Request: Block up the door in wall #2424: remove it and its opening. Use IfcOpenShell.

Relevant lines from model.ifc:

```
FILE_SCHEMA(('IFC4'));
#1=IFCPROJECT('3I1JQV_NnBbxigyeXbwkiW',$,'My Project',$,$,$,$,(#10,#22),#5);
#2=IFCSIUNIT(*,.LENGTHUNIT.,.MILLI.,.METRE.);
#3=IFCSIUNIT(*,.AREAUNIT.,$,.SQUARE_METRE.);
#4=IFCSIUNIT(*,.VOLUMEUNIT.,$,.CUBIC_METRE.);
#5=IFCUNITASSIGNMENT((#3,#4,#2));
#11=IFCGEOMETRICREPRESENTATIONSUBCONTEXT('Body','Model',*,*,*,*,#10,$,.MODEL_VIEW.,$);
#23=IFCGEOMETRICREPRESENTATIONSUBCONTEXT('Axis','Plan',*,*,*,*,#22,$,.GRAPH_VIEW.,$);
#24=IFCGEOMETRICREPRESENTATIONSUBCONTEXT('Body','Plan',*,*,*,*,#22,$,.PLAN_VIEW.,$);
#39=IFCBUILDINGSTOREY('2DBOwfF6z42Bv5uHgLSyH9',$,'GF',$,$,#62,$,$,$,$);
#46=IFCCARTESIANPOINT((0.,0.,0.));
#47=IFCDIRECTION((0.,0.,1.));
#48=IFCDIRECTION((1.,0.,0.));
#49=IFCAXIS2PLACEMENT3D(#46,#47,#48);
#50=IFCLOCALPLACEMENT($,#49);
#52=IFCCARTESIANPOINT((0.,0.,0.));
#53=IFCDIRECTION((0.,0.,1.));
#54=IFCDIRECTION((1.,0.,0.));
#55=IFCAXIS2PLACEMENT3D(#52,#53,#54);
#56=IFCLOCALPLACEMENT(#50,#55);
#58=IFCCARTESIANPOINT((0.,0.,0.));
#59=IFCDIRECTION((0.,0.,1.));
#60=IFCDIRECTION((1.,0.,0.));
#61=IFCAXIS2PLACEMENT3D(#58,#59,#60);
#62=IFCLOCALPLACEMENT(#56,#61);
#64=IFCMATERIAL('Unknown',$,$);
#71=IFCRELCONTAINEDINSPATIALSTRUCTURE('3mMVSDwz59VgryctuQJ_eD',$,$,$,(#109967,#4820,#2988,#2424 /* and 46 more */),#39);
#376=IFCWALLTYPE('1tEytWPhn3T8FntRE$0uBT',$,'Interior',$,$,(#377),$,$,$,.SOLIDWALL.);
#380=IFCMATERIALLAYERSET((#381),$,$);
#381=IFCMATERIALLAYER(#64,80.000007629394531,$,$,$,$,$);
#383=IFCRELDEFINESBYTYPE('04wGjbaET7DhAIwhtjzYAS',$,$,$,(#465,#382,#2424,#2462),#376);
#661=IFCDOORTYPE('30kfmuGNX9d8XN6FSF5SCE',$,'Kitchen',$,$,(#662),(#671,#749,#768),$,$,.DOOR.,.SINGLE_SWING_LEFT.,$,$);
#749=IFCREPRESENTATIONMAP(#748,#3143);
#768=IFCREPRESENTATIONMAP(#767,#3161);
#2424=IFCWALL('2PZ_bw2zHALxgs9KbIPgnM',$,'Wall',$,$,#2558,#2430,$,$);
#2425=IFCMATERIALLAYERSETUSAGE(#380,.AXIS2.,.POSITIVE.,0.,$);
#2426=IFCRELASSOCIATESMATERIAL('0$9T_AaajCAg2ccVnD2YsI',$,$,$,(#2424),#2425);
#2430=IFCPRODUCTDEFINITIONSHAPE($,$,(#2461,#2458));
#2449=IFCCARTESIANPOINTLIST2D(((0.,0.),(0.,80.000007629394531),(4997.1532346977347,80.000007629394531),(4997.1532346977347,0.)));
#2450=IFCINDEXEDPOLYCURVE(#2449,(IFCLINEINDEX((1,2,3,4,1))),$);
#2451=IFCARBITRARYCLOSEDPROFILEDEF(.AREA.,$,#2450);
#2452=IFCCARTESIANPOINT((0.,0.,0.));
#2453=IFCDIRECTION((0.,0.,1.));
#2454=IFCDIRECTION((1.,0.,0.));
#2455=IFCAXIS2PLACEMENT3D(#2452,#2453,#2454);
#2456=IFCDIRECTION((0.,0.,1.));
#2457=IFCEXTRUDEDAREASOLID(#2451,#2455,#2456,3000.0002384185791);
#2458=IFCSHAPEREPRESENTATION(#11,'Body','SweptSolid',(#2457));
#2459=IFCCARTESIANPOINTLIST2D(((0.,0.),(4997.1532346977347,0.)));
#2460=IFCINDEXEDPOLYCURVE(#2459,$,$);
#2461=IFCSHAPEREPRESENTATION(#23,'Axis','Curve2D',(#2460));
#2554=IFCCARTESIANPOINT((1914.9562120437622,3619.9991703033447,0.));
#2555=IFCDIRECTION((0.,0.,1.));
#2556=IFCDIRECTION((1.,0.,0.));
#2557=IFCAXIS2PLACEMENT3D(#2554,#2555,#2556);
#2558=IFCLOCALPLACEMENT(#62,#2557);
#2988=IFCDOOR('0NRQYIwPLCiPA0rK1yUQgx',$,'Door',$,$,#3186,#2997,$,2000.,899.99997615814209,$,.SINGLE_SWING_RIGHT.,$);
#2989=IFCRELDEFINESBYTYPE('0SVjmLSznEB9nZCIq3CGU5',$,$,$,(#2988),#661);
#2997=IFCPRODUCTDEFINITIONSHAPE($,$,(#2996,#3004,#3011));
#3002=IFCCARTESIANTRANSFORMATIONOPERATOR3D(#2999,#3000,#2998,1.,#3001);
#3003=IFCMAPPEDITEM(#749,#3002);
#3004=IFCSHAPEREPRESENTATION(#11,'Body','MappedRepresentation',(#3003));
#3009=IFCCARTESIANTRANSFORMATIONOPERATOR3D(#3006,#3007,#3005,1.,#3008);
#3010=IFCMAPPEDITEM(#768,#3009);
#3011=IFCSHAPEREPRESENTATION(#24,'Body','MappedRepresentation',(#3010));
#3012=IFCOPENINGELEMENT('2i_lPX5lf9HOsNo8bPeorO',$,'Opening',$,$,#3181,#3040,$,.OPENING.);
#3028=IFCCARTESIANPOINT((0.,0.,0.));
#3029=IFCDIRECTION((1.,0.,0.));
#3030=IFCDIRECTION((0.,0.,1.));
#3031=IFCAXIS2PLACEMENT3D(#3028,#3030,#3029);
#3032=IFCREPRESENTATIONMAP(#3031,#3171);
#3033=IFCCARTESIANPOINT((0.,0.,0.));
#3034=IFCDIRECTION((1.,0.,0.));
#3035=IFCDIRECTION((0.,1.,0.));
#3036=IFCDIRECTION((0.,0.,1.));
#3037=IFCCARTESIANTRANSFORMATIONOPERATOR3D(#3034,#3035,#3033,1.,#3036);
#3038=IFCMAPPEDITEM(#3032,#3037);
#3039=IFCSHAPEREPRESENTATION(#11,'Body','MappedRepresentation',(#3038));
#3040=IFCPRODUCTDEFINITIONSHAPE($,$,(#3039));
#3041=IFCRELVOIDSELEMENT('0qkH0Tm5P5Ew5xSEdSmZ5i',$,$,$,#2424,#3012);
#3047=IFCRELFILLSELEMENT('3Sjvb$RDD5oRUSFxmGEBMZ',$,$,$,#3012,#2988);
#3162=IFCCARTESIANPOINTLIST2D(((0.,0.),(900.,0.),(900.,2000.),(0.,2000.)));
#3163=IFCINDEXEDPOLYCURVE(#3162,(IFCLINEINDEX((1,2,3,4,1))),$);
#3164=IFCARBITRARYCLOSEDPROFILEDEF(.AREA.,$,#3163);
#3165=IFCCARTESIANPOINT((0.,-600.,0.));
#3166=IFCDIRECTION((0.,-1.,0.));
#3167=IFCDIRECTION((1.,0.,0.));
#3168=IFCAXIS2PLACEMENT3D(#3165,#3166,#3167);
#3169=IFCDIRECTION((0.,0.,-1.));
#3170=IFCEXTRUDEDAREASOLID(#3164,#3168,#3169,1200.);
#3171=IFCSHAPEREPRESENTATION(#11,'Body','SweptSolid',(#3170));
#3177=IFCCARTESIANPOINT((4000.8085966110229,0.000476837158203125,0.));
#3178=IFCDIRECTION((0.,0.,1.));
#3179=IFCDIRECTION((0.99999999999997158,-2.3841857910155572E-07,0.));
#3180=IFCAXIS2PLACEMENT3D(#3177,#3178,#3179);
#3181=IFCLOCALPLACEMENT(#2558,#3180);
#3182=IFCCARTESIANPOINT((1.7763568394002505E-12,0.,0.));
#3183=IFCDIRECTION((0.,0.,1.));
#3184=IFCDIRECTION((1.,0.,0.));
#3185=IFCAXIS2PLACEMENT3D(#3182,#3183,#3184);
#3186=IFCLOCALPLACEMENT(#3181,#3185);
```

```python
import ifcopenshell
import ifcopenshell.api.feature
import ifcopenshell.api.root
import ifcopenshell.geom
import ifcopenshell.util.shape

model = ifcopenshell.open("model.ifc")
settings = ifcopenshell.geom.settings()


def volume(element):
    """Net volume in cubic metres, openings subtracted."""
    shape = ifcopenshell.geom.create_shape(settings, element)
    return ifcopenshell.util.shape.get_volume(shape.geometry)


door = model.by_id(2988)
opening = door.FillsVoids[0].RelatingOpeningElement
wall = opening.VoidsElements[0].RelatingBuildingElement
before = volume(wall)

ifcopenshell.api.root.remove_product(model, product=door)
ifcopenshell.api.feature.remove_feature(model, feature=opening)

after = volume(wall)

print(f"wall volume {before:.3f} -> {after:.3f} m3")

model.write("model_v2.ifc")
```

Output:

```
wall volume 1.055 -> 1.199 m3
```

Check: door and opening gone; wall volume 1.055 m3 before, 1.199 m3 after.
